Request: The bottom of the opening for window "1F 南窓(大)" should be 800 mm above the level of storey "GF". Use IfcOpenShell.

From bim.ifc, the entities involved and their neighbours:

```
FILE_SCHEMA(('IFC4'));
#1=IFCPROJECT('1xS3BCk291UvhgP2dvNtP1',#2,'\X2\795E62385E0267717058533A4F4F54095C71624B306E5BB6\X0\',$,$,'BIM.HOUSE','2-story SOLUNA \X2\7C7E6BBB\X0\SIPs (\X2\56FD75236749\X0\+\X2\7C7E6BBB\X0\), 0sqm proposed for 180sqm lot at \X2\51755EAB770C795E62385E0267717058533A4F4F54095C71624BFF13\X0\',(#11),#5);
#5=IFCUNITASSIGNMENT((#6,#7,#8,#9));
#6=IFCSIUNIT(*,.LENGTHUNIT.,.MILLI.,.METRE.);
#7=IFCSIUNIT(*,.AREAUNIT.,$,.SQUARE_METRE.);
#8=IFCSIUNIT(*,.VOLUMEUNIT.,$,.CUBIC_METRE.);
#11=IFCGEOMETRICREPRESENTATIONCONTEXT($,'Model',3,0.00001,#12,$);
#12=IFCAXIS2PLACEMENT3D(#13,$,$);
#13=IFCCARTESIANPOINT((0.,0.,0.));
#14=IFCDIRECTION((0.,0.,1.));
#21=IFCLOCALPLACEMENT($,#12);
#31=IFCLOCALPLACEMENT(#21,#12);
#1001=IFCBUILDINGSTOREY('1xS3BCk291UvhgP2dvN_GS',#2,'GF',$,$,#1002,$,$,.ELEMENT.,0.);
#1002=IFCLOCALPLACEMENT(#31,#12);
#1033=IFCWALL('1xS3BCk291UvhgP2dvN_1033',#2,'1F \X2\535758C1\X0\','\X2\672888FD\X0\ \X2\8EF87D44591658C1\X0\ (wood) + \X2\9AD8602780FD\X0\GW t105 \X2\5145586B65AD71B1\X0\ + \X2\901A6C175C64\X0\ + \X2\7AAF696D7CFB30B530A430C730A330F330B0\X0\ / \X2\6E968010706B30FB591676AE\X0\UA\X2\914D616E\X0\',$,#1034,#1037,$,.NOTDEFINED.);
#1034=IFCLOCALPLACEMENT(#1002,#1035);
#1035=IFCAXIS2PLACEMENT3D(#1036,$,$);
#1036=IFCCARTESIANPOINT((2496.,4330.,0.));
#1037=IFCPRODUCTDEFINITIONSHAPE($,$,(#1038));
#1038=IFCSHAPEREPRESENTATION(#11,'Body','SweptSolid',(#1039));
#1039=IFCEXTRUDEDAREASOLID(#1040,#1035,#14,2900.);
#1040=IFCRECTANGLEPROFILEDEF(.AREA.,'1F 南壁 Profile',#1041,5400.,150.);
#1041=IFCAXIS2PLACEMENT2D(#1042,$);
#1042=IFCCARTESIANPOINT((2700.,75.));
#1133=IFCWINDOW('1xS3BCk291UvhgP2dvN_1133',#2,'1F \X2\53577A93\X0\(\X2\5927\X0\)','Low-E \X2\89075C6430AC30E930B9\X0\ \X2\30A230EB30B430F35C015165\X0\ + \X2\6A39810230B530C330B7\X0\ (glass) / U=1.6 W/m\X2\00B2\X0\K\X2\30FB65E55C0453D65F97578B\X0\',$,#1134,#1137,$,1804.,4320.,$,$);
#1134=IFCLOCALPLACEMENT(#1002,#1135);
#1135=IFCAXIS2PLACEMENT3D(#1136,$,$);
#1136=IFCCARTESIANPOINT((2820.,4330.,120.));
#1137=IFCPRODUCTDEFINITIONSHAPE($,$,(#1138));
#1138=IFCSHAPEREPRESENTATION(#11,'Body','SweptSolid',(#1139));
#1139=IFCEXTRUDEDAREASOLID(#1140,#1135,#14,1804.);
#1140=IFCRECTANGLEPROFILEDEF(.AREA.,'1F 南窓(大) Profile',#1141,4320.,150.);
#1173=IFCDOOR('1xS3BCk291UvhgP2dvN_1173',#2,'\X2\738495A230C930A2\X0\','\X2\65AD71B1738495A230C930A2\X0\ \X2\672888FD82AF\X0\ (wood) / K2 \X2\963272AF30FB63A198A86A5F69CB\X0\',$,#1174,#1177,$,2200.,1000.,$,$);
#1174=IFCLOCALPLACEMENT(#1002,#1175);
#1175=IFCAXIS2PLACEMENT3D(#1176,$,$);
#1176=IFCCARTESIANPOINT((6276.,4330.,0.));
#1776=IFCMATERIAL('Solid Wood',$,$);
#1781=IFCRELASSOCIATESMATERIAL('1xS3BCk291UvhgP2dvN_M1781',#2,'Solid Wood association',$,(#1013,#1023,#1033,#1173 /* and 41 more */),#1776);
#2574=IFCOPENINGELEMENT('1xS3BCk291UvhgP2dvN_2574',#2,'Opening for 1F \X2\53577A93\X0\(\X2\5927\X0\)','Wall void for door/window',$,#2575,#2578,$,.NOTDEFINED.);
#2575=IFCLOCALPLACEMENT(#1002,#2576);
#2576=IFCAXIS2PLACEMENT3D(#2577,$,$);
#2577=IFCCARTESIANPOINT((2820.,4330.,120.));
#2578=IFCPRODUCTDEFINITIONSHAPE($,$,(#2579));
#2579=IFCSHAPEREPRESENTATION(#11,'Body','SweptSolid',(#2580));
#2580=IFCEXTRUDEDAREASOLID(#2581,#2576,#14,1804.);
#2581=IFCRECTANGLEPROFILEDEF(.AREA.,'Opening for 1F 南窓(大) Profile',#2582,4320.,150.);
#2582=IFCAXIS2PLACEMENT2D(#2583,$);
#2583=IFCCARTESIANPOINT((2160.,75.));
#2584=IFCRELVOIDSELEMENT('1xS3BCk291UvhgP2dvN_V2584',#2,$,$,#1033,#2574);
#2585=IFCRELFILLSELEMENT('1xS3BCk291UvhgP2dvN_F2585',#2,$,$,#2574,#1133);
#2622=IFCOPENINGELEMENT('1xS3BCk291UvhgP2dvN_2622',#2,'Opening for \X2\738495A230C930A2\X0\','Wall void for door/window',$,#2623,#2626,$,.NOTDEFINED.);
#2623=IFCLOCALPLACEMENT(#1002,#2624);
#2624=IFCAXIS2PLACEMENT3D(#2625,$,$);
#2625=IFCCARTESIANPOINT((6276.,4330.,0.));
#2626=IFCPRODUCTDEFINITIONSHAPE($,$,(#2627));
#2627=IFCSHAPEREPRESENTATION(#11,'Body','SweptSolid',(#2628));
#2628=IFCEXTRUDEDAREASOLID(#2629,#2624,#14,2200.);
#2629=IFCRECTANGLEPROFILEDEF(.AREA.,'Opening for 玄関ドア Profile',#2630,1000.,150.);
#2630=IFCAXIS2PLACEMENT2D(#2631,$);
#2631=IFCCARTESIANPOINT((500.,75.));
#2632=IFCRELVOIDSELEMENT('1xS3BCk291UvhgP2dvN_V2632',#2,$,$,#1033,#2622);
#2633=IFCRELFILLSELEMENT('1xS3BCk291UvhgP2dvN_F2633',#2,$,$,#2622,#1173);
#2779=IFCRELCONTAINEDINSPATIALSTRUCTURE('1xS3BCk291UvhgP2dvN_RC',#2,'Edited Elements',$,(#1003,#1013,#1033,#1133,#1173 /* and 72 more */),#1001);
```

```python
import numpy as np
import ifcopenshell
import ifcopenshell.api.geometry
import ifcopenshell.geom
import ifcopenshell.util.element
import ifcopenshell.util.placement
import ifcopenshell.util.shape
import ifcopenshell.util.unit

model = ifcopenshell.open("bim.ifc")
unit_scale = ifcopenshell.util.unit.calculate_unit_scale(model)

window = model.by_id(1133)
opening = window.FillsVoids[0].RelatingOpeningElement
storey = ifcopenshell.util.element.get_container(window, ifc_class="IfcBuildingStorey")
level = ifcopenshell.util.placement.get_local_placement(storey.ObjectPlacement)[2, 3]

# The opening's origin need not be at the sill, so measure its lowest point.
shape = ifcopenshell.geom.create_shape(ifcopenshell.geom.settings(), opening)
bottom = ifcopenshell.util.shape.get_shape_bottom_elevation(shape, shape.geometry) / unit_scale
dz = level + 0.8 / unit_scale - bottom

shift = np.array([0.0, 0.0, dz])
# The window is not placed relative to its opening, so move both.
for product in (opening, window):
    matrix = ifcopenshell.util.placement.get_local_placement(product.ObjectPlacement)
    matrix[:3, 3] += shift
    ifcopenshell.api.geometry.edit_object_placement(model, product=product, matrix=matrix, is_si=False)

print(f"moved by {dz * unit_scale:+.3f} m")

model.write("bim_edited.ifc")
```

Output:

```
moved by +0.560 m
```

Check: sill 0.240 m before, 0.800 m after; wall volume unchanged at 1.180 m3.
